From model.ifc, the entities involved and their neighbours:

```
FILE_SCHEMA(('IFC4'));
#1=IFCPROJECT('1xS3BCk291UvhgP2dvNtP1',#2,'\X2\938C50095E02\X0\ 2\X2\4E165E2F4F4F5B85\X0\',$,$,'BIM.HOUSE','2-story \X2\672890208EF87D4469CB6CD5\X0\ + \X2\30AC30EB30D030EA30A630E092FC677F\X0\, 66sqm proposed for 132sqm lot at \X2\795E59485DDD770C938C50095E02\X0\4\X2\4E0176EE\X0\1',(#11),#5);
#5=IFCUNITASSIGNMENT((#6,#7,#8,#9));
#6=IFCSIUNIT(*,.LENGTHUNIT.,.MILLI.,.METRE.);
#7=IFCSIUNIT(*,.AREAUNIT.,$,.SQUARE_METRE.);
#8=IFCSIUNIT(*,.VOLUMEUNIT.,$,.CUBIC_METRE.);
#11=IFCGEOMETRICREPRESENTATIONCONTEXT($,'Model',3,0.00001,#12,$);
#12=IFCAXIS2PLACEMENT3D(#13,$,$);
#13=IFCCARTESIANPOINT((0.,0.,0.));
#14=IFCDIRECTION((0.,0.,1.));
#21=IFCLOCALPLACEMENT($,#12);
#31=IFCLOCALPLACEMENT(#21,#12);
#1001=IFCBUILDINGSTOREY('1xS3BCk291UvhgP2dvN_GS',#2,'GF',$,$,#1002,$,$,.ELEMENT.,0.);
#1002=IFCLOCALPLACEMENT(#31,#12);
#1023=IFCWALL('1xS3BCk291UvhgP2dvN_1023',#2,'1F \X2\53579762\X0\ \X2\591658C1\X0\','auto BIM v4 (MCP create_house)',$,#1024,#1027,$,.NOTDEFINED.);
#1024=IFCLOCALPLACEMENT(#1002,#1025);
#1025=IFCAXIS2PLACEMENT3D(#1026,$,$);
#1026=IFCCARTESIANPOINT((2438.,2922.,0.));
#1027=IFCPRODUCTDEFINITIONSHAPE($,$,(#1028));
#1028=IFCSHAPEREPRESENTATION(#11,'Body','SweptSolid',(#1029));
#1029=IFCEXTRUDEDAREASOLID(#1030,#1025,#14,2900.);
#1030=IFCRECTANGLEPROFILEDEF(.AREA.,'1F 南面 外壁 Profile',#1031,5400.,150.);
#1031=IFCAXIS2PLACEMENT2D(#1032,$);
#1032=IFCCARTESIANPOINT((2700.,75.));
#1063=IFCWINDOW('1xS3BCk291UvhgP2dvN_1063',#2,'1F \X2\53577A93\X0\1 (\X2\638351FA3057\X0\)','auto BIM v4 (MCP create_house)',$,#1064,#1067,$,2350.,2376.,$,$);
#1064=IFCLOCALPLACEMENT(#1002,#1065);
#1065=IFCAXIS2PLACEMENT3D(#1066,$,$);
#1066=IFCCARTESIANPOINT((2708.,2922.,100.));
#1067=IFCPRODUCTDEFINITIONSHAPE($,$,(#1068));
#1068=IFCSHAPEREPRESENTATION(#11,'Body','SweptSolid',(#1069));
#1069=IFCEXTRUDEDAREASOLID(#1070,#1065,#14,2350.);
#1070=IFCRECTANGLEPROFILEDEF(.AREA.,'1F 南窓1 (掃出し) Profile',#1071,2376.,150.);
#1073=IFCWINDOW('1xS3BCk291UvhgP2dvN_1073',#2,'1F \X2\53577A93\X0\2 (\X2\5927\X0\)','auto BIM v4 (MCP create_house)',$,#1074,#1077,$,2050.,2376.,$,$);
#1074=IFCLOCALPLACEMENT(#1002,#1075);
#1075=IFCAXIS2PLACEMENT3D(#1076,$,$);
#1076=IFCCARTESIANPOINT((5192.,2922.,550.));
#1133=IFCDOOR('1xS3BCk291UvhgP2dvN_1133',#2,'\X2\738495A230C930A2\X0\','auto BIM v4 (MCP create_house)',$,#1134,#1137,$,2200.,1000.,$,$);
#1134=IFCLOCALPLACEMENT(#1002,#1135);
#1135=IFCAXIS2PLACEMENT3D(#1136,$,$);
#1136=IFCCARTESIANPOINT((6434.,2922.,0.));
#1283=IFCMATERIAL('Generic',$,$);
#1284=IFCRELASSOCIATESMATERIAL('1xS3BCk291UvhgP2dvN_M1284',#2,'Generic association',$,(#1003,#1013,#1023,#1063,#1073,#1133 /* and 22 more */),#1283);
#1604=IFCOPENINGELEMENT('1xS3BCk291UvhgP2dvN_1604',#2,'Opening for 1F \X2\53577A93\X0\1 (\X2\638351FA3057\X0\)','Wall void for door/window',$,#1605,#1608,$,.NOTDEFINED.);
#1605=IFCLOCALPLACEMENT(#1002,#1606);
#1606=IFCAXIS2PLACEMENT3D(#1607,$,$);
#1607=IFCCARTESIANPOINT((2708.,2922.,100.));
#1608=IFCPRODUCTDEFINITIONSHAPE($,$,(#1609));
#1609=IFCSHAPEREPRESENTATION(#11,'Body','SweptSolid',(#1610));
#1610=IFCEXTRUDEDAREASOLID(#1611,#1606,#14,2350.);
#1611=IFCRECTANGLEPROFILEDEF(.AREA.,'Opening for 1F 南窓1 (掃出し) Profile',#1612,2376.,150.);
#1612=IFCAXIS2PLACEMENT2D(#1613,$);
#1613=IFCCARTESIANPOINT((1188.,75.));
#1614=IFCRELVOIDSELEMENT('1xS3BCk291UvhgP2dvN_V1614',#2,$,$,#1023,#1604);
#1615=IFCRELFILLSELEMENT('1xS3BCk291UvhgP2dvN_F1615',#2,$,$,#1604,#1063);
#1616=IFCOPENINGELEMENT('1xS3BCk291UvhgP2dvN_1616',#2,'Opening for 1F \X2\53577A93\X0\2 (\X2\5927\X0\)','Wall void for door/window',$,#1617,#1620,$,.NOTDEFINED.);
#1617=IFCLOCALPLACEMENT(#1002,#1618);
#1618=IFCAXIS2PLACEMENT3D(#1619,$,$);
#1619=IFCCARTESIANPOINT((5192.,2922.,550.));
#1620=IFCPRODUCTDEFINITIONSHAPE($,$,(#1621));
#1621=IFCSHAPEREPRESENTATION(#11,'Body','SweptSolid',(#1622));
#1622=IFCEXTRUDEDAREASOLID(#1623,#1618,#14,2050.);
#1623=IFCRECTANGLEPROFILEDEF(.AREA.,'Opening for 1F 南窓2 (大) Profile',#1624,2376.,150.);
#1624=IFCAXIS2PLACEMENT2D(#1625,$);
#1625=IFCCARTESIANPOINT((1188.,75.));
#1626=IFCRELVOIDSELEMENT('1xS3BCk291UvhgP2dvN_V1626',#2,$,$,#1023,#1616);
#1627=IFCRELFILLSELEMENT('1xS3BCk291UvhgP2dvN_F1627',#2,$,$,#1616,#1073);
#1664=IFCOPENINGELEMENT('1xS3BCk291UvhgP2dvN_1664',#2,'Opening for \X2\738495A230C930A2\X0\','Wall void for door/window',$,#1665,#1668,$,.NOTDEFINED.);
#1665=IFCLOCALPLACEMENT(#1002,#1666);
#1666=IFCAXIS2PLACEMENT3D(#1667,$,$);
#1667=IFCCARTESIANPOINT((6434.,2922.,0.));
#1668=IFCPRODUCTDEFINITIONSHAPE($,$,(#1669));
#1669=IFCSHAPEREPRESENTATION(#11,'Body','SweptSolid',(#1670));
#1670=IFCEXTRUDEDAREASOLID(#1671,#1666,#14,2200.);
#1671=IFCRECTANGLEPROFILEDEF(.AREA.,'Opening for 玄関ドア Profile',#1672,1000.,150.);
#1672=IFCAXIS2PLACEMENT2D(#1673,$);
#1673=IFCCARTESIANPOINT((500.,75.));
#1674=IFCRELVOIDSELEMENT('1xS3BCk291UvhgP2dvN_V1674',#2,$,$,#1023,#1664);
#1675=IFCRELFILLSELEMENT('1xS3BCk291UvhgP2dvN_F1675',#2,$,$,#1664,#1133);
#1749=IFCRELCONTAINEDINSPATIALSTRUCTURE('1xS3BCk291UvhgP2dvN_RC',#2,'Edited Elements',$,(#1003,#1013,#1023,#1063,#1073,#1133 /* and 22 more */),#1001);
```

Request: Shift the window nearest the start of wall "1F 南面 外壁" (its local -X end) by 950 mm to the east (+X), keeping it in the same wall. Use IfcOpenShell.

```python
import ifcopenshell
import ifcopenshell.api.geometry
import ifcopenshell.util.placement

model = ifcopenshell.open("model.ifc")

window = model.by_guid("1xS3BCk291UvhgP2dvN_1063")
opening = window.FillsVoids[0].RelatingOpeningElement
wall = opening.VoidsElements[0].RelatingBuildingElement

wall_matrix = ifcopenshell.util.placement.get_local_placement(wall.ObjectPlacement)
shift = wall_matrix[:3, 0] * 950.0
before = ifcopenshell.util.placement.get_local_placement(window.ObjectPlacement)[:3, 3].copy()

# The window is not placed relative to its opening, so move both.
for product in (opening, window):
    matrix = ifcopenshell.util.placement.get_local_placement(product.ObjectPlacement)
    matrix[:3, 3] += shift
    ifcopenshell.api.geometry.edit_object_placement(model, product=product, matrix=matrix, is_si=False)

after = ifcopenshell.util.placement.get_local_placement(window.ObjectPlacement)[:3, 3]
print("window moved by", (after - before).round(3) + 0.0)

model.write("model_rev.ifc")
```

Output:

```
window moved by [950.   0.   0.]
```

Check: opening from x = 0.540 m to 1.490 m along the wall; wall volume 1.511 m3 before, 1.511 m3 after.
